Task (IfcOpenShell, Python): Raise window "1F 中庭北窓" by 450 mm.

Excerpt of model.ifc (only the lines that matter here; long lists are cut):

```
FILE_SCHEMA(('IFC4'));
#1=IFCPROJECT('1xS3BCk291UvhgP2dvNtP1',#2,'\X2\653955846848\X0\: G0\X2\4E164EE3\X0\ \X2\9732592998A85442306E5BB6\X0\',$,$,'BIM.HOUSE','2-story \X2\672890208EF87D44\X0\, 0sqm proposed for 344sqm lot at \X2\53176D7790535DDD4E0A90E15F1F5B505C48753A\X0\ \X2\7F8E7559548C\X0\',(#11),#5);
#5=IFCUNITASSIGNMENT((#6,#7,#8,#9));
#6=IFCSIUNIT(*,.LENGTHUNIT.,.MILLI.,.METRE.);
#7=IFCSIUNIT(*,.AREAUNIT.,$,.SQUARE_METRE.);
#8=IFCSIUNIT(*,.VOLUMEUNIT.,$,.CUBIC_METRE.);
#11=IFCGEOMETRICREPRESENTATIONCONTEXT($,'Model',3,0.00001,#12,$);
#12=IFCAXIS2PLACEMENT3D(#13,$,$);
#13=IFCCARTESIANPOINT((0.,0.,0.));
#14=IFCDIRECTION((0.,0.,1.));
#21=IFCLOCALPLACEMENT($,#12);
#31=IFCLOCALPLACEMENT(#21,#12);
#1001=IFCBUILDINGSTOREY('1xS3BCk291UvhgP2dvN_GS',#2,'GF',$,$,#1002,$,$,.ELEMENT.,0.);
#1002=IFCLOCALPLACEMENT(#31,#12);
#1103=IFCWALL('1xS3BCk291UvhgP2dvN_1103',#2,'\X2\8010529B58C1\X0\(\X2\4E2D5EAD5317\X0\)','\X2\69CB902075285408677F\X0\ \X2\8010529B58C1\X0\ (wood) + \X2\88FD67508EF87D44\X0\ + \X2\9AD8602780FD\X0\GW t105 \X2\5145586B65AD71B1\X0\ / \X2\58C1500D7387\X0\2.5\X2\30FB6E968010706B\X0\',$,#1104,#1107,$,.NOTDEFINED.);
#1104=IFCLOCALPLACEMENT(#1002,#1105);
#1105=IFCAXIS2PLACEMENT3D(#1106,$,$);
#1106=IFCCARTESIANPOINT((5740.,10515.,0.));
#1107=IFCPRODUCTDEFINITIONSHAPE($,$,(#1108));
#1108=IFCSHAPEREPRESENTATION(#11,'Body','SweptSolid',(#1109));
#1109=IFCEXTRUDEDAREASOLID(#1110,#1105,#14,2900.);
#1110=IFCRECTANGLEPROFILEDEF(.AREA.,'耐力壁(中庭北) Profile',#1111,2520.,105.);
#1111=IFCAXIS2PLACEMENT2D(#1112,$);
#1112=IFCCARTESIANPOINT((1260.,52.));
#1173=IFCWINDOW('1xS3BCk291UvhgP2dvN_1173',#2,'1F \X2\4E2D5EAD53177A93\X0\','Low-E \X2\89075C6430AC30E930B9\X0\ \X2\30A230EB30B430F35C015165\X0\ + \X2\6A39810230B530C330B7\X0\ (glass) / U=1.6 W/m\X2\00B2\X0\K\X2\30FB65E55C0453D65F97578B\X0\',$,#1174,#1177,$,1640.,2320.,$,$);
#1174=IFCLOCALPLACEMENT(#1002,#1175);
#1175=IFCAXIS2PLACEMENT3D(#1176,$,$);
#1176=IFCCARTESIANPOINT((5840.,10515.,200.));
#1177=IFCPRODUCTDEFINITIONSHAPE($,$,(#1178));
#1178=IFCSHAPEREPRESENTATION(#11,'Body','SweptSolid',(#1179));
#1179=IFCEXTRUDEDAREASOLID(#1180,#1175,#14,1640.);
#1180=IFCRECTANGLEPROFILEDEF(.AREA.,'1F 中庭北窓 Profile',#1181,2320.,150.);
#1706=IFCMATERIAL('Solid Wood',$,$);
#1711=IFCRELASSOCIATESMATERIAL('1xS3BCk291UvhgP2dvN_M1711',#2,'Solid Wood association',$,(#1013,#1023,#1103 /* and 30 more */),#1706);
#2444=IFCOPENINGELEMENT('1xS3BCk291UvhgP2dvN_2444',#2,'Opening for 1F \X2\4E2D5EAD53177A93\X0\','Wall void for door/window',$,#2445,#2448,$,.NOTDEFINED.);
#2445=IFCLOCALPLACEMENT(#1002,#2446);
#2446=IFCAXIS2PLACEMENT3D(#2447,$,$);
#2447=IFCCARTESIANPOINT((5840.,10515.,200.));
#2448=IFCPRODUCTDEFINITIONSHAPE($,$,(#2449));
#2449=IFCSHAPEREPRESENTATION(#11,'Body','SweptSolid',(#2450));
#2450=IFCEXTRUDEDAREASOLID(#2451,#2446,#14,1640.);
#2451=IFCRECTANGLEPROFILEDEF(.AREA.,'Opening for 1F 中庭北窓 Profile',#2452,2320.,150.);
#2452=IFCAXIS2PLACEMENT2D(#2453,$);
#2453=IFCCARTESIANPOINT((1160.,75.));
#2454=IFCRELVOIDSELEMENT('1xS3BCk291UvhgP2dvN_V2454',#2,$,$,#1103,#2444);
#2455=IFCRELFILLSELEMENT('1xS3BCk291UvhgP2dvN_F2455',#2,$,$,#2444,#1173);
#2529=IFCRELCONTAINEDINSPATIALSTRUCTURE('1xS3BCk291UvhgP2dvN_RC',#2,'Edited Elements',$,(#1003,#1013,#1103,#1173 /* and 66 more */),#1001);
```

```python
import numpy as np
import ifcopenshell
import ifcopenshell.api.geometry
import ifcopenshell.util.placement
import ifcopenshell.util.unit

model = ifcopenshell.open("model.ifc")
unit_scale = ifcopenshell.util.unit.calculate_unit_scale(model)

window = model.by_guid("1xS3BCk291UvhgP2dvN_1173")
opening = window.FillsVoids[0].RelatingOpeningElement
dz = 0.45 / unit_scale

shift = np.array([0.0, 0.0, dz])
# The window is not placed relative to its opening, so move both.
for product in (opening, window):
    matrix = ifcopenshell.util.placement.get_local_placement(product.ObjectPlacement)
    matrix[:3, 3] += shift
    ifcopenshell.api.geometry.edit_object_placement(model, product=product, matrix=matrix, is_si=False)

print(f"moved by {dz * unit_scale:+.3f} m")

model.write("model-out.ifc")
```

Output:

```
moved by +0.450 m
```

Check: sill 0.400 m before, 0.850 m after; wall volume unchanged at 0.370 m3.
